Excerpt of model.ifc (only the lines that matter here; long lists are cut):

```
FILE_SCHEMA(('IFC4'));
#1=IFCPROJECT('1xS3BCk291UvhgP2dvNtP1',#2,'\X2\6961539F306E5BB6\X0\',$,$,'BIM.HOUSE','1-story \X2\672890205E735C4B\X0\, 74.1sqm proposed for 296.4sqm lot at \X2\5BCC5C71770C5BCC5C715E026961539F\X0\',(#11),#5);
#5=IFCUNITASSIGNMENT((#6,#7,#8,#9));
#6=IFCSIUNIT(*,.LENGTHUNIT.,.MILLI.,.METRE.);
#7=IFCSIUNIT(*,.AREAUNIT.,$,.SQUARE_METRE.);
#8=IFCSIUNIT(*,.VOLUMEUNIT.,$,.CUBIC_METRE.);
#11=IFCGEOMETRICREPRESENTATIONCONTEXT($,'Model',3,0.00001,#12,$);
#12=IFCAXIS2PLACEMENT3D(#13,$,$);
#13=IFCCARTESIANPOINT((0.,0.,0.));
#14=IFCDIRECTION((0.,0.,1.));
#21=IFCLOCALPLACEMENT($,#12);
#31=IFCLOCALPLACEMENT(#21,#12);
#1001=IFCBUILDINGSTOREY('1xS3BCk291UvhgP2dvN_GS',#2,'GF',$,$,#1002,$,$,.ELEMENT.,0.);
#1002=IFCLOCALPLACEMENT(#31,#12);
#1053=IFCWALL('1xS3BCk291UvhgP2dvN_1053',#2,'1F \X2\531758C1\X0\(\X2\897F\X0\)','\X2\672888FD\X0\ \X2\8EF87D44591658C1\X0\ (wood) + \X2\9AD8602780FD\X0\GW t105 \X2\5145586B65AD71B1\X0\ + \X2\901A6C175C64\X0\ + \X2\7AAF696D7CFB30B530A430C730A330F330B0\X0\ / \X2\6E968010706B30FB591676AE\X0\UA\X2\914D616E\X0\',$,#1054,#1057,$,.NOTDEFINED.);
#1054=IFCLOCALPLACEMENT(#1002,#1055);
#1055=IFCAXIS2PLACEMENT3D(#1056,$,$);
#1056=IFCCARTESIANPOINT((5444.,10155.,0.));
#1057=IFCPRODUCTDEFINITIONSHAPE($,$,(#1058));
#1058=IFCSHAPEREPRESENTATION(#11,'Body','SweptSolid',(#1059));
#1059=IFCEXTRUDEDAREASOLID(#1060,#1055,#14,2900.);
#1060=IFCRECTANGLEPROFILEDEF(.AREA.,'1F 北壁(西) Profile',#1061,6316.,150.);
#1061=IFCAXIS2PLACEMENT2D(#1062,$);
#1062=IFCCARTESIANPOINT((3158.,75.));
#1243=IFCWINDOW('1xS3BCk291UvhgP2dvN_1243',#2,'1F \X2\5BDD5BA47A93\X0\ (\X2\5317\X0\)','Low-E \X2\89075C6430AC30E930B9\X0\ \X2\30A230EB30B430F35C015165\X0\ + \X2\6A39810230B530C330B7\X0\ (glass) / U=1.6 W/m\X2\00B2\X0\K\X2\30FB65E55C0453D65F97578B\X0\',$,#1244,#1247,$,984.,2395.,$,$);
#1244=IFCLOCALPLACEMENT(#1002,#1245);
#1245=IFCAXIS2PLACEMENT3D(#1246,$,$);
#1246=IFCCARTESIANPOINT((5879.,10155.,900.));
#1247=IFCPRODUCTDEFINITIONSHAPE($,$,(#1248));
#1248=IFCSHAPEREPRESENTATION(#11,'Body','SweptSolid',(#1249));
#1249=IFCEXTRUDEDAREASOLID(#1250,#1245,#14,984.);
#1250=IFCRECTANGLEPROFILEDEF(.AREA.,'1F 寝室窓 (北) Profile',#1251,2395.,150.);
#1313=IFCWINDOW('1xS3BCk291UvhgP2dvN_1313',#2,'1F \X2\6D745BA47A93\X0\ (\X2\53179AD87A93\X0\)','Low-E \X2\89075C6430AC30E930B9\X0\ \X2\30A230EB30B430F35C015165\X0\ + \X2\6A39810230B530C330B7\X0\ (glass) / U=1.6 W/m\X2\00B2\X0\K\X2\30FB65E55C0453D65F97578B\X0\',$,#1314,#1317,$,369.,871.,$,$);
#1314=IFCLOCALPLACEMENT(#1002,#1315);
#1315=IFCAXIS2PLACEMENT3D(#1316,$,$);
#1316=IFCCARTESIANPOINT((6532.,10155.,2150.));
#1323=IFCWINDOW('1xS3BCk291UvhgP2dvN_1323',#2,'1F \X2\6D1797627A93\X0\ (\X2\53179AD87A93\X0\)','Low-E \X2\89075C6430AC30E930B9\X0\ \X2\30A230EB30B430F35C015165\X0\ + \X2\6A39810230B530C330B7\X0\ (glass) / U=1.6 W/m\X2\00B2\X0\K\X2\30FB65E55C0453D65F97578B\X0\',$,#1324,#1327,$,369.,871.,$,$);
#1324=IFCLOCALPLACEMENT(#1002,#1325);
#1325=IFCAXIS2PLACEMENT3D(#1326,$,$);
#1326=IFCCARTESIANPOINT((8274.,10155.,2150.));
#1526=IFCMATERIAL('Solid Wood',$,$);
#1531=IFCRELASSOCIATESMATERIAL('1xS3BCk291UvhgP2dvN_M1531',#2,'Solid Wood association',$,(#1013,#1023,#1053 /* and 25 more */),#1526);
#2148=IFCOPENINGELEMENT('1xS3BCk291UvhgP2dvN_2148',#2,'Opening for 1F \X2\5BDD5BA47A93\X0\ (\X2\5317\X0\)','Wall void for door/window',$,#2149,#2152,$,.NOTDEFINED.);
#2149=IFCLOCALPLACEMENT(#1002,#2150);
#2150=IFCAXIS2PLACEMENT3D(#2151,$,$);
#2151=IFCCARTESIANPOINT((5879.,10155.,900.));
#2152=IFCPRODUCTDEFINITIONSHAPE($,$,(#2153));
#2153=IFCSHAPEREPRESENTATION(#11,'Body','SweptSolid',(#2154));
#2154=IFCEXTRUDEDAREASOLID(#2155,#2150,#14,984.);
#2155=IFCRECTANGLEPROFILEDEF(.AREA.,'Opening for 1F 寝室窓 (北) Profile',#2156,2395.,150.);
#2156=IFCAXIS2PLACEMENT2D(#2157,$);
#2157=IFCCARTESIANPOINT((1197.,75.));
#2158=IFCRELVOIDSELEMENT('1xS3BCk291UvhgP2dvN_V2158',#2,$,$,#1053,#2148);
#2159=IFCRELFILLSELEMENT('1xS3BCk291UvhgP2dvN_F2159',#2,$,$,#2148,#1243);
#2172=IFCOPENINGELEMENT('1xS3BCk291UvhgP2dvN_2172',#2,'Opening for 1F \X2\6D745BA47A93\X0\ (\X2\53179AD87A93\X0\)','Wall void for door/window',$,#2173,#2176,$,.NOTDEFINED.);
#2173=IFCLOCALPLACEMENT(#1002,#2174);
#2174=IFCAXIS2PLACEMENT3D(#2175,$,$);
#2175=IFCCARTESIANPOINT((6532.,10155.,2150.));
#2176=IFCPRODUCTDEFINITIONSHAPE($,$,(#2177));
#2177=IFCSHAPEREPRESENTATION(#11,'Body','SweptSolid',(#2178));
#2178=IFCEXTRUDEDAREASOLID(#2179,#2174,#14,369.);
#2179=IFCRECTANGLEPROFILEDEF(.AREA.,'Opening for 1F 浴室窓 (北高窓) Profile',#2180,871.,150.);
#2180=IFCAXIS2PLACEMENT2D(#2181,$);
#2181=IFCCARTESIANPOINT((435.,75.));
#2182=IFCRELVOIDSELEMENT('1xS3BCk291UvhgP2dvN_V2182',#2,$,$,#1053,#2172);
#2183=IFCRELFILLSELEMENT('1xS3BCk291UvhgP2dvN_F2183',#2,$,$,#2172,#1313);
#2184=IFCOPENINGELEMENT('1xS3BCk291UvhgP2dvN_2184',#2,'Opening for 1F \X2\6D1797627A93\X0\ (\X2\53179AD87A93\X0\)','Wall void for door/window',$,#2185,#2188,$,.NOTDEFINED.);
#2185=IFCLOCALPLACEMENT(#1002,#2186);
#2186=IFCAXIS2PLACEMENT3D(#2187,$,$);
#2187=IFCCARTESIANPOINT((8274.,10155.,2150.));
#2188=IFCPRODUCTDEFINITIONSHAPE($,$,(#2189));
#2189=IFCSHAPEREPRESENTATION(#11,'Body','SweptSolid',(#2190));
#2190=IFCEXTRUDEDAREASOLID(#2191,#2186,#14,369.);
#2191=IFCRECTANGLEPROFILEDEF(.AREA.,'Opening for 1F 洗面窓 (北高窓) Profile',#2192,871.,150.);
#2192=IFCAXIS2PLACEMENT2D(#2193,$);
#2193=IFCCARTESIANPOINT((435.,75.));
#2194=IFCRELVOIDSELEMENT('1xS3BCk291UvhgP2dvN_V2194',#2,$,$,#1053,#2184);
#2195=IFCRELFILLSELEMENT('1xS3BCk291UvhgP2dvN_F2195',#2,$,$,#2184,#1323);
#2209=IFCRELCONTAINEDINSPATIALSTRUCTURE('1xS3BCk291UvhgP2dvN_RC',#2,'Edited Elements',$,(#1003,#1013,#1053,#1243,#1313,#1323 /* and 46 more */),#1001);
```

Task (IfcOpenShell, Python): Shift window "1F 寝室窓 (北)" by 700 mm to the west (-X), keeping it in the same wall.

```python
import ifcopenshell
import ifcopenshell.api.geometry
import ifcopenshell.util.placement

model = ifcopenshell.open("model.ifc")

window = model.by_id(1243)
opening = window.FillsVoids[0].RelatingOpeningElement
wall = opening.VoidsElements[0].RelatingBuildingElement

wall_matrix = ifcopenshell.util.placement.get_local_placement(wall.ObjectPlacement)
shift = wall_matrix[:3, 0] * -700.0
before = ifcopenshell.util.placement.get_local_placement(window.ObjectPlacement)[:3, 3].copy()

# The window is not placed relative to its opening, so move both.
for product in (opening, window):
    matrix = ifcopenshell.util.placement.get_local_placement(product.ObjectPlacement)
    matrix[:3, 3] += shift
    ifcopenshell.api.geometry.edit_object_placement(model, product=product, matrix=matrix, is_si=False)

after = ifcopenshell.util.placement.get_local_placement(window.ObjectPlacement)[:3, 3]
print("window moved by", (after - before).round(3) + 0.0)

model.write("model-out.ifc")
```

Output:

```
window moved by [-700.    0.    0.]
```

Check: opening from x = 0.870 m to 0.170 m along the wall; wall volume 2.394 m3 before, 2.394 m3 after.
